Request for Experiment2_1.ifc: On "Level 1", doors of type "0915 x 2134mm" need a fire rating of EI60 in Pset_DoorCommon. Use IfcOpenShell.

First a look at what the model holds.

```python
import ifcopenshell
import ifcopenshell.util.element

model = ifcopenshell.open("Experiment2_1.ifc")
print(model.schema)
storey = next(s for s in model.by_type("IfcBuildingStorey") if s.Name == "Level 1")
doors = [e for e in ifcopenshell.util.element.get_decomposition(storey) if e.is_a("IfcDoor")]
seen = {}
for e in doors:
    element_type = ifcopenshell.util.element.get_type(e)
    key = (element_type.Name if element_type != e and element_type else None, ifcopenshell.util.element.get_pset(e, "Pset_DoorCommon", "FireRating"))
    seen[key] = seen.get(key, 0) + 1
for (name, value), count in sorted(seen.items(), key=str):
    print(count, "x", name, "|", value)
```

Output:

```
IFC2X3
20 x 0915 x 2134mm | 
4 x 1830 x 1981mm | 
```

```python
import ifcopenshell
import ifcopenshell.api.pset
import ifcopenshell.util.element

model = ifcopenshell.open("Experiment2_1.ifc")

storey = next(s for s in model.by_type("IfcBuildingStorey") if s.Name == "Level 1")
doors = [e for e in ifcopenshell.util.element.get_decomposition(storey) if e.is_a("IfcDoor")]

count = 0
for e in doors:
    element_type = ifcopenshell.util.element.get_type(e)
    if element_type in (None, e) or element_type.Name != "0915 x 2134mm":
        continue
    # add_pset returns the element's existing set when there is one.
    pset = ifcopenshell.api.pset.add_pset(model, product=e, name="Pset_DoorCommon")
    ifcopenshell.api.pset.edit_pset(model, pset=pset, properties={"FireRating": "EI60"})
    count += 1

print(count, "doors updated")

model.write("Experiment2_1_edited.ifc")
```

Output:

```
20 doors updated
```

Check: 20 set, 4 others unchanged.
